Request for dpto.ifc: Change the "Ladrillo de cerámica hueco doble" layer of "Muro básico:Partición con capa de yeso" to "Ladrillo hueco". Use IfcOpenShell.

First a look at what the model holds.

```python
import ifcopenshell
import ifcopenshell.util.element

model = ifcopenshell.open("dpto.ifc")
print(model.schema)
for layer_set in model.by_type("IfcMaterialLayerSet"):
    if layer_set.LayerSetName == "Muro básico:Partición con capa de yeso":
        for layer in layer_set.MaterialLayers:
            print(layer.id(), layer.Material and layer.Material.Name, layer.LayerThickness, sep=" | ")
        print(len(ifcopenshell.util.element.get_elements_by_material(model, layer_set)), "elements and types use it")
print(sorted(m.Name for m in model.by_type("IfcMaterial") if m.Name)[:60])
```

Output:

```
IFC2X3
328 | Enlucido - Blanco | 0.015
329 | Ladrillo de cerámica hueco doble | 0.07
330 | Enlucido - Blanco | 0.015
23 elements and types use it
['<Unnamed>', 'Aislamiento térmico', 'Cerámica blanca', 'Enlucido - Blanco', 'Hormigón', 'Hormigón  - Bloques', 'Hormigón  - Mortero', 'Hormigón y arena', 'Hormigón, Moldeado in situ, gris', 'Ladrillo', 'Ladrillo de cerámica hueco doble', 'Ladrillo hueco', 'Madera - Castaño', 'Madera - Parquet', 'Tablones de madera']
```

```python
import ifcopenshell
import ifcopenshell.api.material

model = ifcopenshell.open("dpto.ifc")

layer_set = next(s for s in model.by_type("IfcMaterialLayerSet") if s.LayerSetName == "Muro básico:Partición con capa de yeso")
layer = next(l for l in layer_set.MaterialLayers if l.Material and l.Material.Name == "Ladrillo de cerámica hueco doble")
material = next(m for m in model.by_type("IfcMaterial") if m.Name == "Ladrillo hueco")

# Point this one layer at the other material; renaming the old one would change it everywhere.
ifcopenshell.api.material.edit_layer(model, layer=layer, attributes={}, material=material)

print([l.Material.Name if l.Material else None for l in layer_set.MaterialLayers])

model.write("dpto_edited.ifc")
```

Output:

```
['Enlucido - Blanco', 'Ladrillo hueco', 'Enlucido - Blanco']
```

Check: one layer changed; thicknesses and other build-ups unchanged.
